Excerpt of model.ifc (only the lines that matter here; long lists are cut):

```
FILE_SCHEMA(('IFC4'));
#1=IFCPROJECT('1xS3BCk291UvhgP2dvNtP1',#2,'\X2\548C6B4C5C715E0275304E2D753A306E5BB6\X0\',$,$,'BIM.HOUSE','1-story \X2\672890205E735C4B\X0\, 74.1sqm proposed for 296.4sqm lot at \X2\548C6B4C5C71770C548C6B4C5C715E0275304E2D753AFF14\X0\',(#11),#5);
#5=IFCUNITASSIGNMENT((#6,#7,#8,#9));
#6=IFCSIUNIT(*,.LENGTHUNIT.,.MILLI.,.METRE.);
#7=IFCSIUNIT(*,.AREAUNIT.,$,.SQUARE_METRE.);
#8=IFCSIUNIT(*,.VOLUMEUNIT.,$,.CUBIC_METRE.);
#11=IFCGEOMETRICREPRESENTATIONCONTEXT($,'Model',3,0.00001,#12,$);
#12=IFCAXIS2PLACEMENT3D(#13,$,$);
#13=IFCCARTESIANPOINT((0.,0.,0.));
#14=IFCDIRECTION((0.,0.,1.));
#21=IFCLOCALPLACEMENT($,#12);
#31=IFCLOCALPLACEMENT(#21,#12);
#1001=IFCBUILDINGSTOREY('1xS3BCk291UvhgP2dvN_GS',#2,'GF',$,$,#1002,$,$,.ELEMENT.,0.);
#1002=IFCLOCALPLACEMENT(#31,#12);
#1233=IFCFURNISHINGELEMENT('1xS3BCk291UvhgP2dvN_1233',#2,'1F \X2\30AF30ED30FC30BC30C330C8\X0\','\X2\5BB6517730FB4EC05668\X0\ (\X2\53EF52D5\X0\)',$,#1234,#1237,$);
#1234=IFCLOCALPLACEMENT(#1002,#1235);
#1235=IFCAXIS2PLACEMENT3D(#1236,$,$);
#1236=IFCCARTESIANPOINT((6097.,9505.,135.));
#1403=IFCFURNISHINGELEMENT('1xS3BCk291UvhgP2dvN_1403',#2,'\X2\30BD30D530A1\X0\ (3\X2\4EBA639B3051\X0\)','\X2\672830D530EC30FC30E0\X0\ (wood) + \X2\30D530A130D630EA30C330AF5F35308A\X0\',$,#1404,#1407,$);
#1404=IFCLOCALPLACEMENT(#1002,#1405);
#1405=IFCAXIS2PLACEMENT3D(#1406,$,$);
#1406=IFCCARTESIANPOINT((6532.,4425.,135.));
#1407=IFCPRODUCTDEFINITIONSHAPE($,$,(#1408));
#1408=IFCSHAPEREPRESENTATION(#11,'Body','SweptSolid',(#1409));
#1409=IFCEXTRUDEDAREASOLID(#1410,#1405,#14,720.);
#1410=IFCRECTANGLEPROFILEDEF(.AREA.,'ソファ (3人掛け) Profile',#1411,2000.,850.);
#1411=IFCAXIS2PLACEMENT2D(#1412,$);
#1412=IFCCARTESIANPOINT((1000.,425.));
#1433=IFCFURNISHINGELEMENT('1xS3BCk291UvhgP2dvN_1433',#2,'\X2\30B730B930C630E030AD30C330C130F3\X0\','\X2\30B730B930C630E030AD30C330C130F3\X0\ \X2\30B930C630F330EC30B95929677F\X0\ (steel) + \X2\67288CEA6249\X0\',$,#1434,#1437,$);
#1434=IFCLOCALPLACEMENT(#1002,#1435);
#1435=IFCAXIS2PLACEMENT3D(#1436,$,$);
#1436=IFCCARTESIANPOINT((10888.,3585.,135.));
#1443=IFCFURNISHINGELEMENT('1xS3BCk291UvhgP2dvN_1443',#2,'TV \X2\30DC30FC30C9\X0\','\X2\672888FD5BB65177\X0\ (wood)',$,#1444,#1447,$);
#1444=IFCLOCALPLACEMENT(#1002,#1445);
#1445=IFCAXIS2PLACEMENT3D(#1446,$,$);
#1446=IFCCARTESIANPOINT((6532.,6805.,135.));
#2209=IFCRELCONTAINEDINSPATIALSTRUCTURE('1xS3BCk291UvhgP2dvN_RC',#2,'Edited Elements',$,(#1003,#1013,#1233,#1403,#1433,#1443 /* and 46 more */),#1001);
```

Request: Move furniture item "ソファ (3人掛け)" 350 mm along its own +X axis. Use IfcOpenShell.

```python
import ifcopenshell
import ifcopenshell.api.geometry
import ifcopenshell.util.placement
import ifcopenshell.util.unit

model = ifcopenshell.open("model.ifc")
unit_scale = ifcopenshell.util.unit.calculate_unit_scale(model)

item = model.by_guid("1xS3BCk291UvhgP2dvN_1403")
matrix = ifcopenshell.util.placement.get_local_placement(item.ObjectPlacement)
matrix[:3, 3] += matrix[:3, 0] * 0.35 / unit_scale
ifcopenshell.api.geometry.edit_object_placement(model, product=item, matrix=matrix, is_si=False)

print(ifcopenshell.util.placement.get_local_placement(item.ObjectPlacement).round(3) + 0.0)

model.write("model_rev.ifc")
```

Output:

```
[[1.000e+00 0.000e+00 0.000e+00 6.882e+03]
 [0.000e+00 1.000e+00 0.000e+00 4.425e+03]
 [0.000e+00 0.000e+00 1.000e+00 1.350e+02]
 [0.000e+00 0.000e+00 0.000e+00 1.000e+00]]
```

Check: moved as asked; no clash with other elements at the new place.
